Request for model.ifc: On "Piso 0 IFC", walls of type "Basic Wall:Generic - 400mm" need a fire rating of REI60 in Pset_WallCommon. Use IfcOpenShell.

First a look at what the model holds.

```python
import ifcopenshell
import ifcopenshell.util.element

model = ifcopenshell.open("model.ifc")
print(model.schema)
storey = next(s for s in model.by_type("IfcBuildingStorey") if s.Name == "Piso 0 IFC")
walls = [e for e in ifcopenshell.util.element.get_decomposition(storey) if e.is_a("IfcWall")]
seen = {}
for e in walls:
    element_type = ifcopenshell.util.element.get_type(e)
    key = (element_type.Name if element_type != e and element_type else None, ifcopenshell.util.element.get_pset(e, "Pset_WallCommon", "FireRating"))
    seen[key] = seen.get(key, 0) + 1
for (name, value), count in sorted(seen.items(), key=str):
    print(count, "x", name, "|", value)
```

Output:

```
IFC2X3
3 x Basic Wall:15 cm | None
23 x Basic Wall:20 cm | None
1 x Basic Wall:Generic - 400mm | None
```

```python
import ifcopenshell
import ifcopenshell.api.pset
import ifcopenshell.util.element

model = ifcopenshell.open("model.ifc")

storey = next(s for s in model.by_type("IfcBuildingStorey") if s.Name == "Piso 0 IFC")
walls = [e for e in ifcopenshell.util.element.get_decomposition(storey) if e.is_a("IfcWall")]

count = 0
for e in walls:
    element_type = ifcopenshell.util.element.get_type(e)
    if element_type in (None, e) or element_type.Name != "Basic Wall:Generic - 400mm":
        continue
    # add_pset returns the element's existing set when there is one.
    pset = ifcopenshell.api.pset.add_pset(model, product=e, name="Pset_WallCommon")
    ifcopenshell.api.pset.edit_pset(model, pset=pset, properties={"FireRating": "REI60"})
    count += 1

print(count, "walls updated")

model.write("model_edited.ifc")
```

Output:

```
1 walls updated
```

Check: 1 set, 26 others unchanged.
